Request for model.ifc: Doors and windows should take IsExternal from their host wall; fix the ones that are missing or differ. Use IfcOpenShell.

First a look at what the model holds.

```python
import ifcopenshell
import ifcopenshell.util.element

model = ifcopenshell.open("model.ifc")
print(model.schema)
seen = {}
for e in model.by_type("IfcDoor") + model.by_type("IfcWindow"):
    if not e.FillsVoids:
        continue
    host = e.FillsVoids[0].RelatingOpeningElement.VoidsElements[0].RelatingBuildingElement
    own = ifcopenshell.util.element.get_pset(e, f"Pset_{e.is_a()[3:].removesuffix('StandardCase')}Common", "IsExternal")
    wall = ifcopenshell.util.element.get_pset(host, "Pset_WallCommon", "IsExternal")
    seen[e.is_a(), own, wall] = seen.get((e.is_a(), own, wall), 0) + 1
for (cls, own, wall), count in sorted(seen.items(), key=str):
    print(count, cls, "IsExternal:", own, "| host wall:", wall)
```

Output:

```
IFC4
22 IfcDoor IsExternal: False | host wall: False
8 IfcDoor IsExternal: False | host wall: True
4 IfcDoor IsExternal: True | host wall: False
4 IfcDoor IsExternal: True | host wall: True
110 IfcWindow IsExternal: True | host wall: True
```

```python
import ifcopenshell
import ifcopenshell.api.pset
import ifcopenshell.util.element

model = ifcopenshell.open("model.ifc")

count = 0
for ifc_class, pset_name in (("IfcDoor", "Pset_DoorCommon"), ("IfcWindow", "Pset_WindowCommon")):
    for e in model.by_type(ifc_class):
        if not e.FillsVoids:
            continue
        host = e.FillsVoids[0].RelatingOpeningElement.VoidsElements[0].RelatingBuildingElement
        external = ifcopenshell.util.element.get_pset(host, "Pset_WallCommon", "IsExternal")
        if external is None or ifcopenshell.util.element.get_pset(e, pset_name, "IsExternal") == external:
            continue
        pset = ifcopenshell.api.pset.add_pset(model, product=e, name=pset_name)
        ifcopenshell.api.pset.edit_pset(model, pset=pset, properties={"IsExternal": external})
        count += 1

print(count, "updated")

model.write("model_v2.ifc")
```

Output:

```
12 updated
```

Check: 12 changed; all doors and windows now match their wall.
